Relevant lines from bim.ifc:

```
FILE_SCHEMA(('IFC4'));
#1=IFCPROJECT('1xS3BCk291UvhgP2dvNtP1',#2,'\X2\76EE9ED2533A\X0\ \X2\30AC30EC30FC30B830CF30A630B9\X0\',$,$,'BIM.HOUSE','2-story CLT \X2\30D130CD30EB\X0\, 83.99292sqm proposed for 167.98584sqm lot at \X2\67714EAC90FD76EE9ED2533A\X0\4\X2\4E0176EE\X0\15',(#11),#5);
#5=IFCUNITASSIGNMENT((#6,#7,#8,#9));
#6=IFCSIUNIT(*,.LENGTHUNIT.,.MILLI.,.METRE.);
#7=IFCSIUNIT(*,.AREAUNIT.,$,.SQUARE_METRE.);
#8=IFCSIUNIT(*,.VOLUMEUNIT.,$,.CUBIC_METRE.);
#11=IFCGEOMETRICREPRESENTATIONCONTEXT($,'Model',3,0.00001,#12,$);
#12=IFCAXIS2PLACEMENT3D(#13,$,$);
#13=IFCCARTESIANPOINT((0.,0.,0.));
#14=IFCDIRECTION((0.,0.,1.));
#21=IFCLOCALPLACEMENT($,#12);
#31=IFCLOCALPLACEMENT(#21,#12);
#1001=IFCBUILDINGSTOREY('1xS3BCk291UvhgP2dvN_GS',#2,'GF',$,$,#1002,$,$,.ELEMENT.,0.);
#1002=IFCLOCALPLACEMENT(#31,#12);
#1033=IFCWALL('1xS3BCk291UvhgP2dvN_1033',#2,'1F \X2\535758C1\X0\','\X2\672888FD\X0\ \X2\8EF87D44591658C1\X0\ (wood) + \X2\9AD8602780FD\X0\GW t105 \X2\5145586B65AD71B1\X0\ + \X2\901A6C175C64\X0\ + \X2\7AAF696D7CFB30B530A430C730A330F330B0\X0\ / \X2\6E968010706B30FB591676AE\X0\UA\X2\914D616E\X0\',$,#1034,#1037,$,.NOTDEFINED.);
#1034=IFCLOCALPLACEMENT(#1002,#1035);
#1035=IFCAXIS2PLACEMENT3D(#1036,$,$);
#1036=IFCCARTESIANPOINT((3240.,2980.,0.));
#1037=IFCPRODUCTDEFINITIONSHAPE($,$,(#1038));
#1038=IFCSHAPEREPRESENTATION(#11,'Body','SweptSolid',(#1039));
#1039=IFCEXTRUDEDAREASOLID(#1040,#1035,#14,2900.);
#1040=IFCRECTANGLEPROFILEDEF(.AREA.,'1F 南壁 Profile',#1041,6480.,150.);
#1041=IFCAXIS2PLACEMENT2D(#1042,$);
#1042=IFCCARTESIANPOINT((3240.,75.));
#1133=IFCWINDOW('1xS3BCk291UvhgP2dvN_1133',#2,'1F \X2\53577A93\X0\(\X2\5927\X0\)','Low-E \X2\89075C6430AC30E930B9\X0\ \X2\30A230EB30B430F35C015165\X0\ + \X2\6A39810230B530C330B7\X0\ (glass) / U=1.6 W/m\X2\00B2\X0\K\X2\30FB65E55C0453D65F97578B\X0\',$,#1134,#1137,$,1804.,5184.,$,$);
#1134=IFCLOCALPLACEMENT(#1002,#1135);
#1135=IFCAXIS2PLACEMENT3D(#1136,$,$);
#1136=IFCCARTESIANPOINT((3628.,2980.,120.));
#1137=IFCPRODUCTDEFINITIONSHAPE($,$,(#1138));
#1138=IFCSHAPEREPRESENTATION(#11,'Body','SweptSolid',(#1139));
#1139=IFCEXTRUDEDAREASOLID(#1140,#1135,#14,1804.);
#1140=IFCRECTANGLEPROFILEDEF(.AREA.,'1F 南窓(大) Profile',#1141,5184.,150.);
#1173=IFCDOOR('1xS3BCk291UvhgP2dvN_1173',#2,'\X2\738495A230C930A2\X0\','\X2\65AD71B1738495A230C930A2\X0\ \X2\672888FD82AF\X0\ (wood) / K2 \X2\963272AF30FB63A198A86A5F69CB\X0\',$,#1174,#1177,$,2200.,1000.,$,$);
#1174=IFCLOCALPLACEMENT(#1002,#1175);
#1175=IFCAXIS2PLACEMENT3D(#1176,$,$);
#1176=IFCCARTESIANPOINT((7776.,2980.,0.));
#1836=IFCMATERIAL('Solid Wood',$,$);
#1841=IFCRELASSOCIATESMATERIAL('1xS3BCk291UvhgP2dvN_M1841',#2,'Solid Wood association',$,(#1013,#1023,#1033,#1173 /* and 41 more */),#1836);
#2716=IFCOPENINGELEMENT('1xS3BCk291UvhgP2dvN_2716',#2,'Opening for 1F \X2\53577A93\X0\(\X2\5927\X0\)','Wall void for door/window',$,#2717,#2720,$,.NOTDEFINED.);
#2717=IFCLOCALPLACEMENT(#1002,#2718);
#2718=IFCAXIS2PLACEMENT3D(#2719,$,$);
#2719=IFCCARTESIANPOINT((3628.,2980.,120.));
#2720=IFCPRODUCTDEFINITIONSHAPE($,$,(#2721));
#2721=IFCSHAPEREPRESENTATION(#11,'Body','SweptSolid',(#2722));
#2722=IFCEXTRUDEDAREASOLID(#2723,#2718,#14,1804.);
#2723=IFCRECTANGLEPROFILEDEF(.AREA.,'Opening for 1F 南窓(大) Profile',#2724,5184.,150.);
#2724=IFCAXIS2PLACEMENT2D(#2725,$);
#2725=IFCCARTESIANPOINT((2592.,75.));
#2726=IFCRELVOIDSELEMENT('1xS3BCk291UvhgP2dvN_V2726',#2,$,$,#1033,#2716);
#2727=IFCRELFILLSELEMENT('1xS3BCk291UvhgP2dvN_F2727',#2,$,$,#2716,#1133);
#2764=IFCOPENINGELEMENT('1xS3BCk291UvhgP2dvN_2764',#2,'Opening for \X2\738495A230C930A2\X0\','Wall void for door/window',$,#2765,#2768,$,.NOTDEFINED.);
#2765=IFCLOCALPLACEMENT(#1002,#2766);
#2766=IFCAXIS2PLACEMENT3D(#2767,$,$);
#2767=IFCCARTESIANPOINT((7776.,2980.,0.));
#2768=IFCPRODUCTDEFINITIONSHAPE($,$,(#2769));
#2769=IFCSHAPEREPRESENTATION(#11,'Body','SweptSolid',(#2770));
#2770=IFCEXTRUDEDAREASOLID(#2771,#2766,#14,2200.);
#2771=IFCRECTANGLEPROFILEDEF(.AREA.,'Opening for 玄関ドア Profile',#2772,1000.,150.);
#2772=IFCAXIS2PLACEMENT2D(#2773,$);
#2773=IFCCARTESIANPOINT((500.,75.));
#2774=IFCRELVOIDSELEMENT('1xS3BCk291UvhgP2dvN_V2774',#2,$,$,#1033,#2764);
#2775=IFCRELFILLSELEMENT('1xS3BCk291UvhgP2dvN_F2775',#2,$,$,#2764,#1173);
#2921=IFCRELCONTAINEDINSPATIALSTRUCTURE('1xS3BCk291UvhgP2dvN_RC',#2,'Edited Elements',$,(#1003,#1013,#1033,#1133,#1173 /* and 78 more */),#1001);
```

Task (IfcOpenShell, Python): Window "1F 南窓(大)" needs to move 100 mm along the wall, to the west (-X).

```python
import ifcopenshell
import ifcopenshell.api.geometry
import ifcopenshell.util.placement
import ifcopenshell.util.unit

model = ifcopenshell.open("bim.ifc")
unit_scale = ifcopenshell.util.unit.calculate_unit_scale(model)

window = model.by_id(1133)
opening = window.FillsVoids[0].RelatingOpeningElement
wall = opening.VoidsElements[0].RelatingBuildingElement

wall_matrix = ifcopenshell.util.placement.get_local_placement(wall.ObjectPlacement)
shift = wall_matrix[:3, 0] * -0.1 / unit_scale
before = ifcopenshell.util.placement.get_local_placement(window.ObjectPlacement)[:3, 3].copy()

# The window is not placed relative to its opening, so move both.
for product in (opening, window):
    matrix = ifcopenshell.util.placement.get_local_placement(product.ObjectPlacement)
    matrix[:3, 3] += shift
    ifcopenshell.api.geometry.edit_object_placement(model, product=product, matrix=matrix, is_si=False)

after = ifcopenshell.util.placement.get_local_placement(window.ObjectPlacement)[:3, 3]
print("window moved by", (after - before).round(3) + 0.0)

model.write("bim_edited.ifc")
```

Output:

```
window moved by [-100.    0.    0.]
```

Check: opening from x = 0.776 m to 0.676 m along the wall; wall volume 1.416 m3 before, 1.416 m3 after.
